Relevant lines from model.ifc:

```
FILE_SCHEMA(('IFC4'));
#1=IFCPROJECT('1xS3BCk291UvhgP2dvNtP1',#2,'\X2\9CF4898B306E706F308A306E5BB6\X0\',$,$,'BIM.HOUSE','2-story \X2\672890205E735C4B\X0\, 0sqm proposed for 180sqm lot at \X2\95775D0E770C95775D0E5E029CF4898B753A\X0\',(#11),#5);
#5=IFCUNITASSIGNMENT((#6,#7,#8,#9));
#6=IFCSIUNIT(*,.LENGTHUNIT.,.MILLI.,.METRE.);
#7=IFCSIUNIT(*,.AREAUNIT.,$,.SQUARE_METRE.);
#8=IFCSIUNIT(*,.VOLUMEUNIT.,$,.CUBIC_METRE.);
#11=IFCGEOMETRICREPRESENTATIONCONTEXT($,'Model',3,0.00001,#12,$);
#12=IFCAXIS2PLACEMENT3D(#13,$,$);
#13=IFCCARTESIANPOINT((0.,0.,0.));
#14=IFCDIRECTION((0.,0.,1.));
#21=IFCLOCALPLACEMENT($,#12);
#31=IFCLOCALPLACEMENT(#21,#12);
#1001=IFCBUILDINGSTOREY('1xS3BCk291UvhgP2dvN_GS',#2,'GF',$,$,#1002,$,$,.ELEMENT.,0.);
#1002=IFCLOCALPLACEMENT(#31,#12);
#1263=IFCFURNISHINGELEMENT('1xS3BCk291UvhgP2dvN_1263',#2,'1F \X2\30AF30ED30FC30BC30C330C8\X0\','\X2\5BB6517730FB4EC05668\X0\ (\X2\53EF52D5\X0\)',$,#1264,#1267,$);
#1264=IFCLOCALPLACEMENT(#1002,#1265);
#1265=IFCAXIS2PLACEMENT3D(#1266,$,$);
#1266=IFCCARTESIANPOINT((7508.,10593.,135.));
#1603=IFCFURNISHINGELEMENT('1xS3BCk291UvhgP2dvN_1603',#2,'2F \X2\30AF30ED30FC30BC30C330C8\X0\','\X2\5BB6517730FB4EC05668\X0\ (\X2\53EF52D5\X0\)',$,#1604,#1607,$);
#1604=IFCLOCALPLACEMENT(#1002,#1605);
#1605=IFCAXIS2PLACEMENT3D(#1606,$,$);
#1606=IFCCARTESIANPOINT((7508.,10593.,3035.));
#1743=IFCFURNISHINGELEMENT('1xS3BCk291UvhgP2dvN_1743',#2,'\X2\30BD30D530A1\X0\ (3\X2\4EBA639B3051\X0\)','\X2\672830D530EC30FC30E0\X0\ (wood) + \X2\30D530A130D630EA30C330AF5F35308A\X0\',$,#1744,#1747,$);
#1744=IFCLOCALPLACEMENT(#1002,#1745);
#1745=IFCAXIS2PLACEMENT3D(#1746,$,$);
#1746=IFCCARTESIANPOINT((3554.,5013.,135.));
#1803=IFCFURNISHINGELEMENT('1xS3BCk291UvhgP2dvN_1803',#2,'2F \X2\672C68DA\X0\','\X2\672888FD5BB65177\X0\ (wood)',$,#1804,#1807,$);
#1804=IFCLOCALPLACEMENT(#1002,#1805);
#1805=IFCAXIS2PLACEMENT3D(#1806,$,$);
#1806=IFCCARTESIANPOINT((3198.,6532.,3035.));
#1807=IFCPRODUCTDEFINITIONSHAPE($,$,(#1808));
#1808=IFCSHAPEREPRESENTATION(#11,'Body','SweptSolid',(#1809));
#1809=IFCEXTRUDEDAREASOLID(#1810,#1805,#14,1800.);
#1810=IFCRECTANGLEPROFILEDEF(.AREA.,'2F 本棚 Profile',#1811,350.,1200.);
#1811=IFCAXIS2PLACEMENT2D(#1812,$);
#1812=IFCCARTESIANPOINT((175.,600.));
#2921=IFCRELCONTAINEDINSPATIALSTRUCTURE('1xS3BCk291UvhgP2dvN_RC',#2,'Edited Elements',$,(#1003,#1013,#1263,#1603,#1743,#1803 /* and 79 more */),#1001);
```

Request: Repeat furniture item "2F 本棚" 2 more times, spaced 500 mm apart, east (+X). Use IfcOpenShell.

```python
import numpy as np
import ifcopenshell
import ifcopenshell.api.geometry
import ifcopenshell.api.root
import ifcopenshell.util.element
import ifcopenshell.util.placement

model = ifcopenshell.open("model.ifc")


def reuse_history(source, copy):
    """copy_class also copies each property set's owner history, people and application; keep the originals."""
    for rel in copy.IsDefinedBy:
        if rel.is_a("IfcRelDefinesByProperties") and (history := rel.RelatingPropertyDefinition.OwnerHistory):
            rel.RelatingPropertyDefinition.OwnerHistory = source.OwnerHistory
            ifcopenshell.util.element.remove_deep2(model, history)


source = model.by_guid("1xS3BCk291UvhgP2dvN_1803")
base = ifcopenshell.util.placement.get_local_placement(source.ObjectPlacement)
step = np.array([1.0, 0.0, 0.0]) * 500.0

for i in range(1, 3):
    copy = ifcopenshell.api.root.copy_class(model, product=source)
    copy.Representation = ifcopenshell.util.element.copy_deep(
        model, source.Representation, exclude=["IfcGeometricRepresentationContext", "IfcRepresentationMap"]
    )
    reuse_history(source, copy)
    matrix = base.copy()
    matrix[:3, 3] += i * step
    print("added at", matrix[:3, 3].round(3) + 0.0)
    ifcopenshell.api.geometry.edit_object_placement(model, product=copy, matrix=matrix, is_si=False)

model.write("model_v2.ifc")
```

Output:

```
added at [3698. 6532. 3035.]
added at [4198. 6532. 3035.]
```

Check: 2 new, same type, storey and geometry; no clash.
